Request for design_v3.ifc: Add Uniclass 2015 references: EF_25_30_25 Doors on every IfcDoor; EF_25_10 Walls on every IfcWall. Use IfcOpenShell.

First a look at what the model holds.

```python
import ifcopenshell

model = ifcopenshell.open("design_v3.ifc")
print(model.schema)
print("classifications:", [c.Name for c in model.by_type("IfcClassification")])
for ifc_class in ("IfcDoor", "IfcRoof", "IfcStair", "IfcWall", "IfcWindow"):
    print(ifc_class, len(model.by_type(ifc_class)))
```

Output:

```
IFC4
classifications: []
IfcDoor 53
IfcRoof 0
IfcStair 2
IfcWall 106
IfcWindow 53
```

```python
import ifcopenshell
import ifcopenshell.api.classification

model = ifcopenshell.open("design_v3.ifc")

system = ifcopenshell.api.classification.add_classification(model, classification="Uniclass 2015")

codes = {
    "IfcDoor": ("EF_25_30_25", "Doors"),
    "IfcWall": ("EF_25_10", "Walls"),
}
for ifc_class, (code, name) in codes.items():
    products = model.by_type(ifc_class)
    ifcopenshell.api.classification.add_reference(
        model, products=products, classification=system, identification=code, name=name
    )
    print(code, len(products))

model.write("design_v3_v2.ifc")
```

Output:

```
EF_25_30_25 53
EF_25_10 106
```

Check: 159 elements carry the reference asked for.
